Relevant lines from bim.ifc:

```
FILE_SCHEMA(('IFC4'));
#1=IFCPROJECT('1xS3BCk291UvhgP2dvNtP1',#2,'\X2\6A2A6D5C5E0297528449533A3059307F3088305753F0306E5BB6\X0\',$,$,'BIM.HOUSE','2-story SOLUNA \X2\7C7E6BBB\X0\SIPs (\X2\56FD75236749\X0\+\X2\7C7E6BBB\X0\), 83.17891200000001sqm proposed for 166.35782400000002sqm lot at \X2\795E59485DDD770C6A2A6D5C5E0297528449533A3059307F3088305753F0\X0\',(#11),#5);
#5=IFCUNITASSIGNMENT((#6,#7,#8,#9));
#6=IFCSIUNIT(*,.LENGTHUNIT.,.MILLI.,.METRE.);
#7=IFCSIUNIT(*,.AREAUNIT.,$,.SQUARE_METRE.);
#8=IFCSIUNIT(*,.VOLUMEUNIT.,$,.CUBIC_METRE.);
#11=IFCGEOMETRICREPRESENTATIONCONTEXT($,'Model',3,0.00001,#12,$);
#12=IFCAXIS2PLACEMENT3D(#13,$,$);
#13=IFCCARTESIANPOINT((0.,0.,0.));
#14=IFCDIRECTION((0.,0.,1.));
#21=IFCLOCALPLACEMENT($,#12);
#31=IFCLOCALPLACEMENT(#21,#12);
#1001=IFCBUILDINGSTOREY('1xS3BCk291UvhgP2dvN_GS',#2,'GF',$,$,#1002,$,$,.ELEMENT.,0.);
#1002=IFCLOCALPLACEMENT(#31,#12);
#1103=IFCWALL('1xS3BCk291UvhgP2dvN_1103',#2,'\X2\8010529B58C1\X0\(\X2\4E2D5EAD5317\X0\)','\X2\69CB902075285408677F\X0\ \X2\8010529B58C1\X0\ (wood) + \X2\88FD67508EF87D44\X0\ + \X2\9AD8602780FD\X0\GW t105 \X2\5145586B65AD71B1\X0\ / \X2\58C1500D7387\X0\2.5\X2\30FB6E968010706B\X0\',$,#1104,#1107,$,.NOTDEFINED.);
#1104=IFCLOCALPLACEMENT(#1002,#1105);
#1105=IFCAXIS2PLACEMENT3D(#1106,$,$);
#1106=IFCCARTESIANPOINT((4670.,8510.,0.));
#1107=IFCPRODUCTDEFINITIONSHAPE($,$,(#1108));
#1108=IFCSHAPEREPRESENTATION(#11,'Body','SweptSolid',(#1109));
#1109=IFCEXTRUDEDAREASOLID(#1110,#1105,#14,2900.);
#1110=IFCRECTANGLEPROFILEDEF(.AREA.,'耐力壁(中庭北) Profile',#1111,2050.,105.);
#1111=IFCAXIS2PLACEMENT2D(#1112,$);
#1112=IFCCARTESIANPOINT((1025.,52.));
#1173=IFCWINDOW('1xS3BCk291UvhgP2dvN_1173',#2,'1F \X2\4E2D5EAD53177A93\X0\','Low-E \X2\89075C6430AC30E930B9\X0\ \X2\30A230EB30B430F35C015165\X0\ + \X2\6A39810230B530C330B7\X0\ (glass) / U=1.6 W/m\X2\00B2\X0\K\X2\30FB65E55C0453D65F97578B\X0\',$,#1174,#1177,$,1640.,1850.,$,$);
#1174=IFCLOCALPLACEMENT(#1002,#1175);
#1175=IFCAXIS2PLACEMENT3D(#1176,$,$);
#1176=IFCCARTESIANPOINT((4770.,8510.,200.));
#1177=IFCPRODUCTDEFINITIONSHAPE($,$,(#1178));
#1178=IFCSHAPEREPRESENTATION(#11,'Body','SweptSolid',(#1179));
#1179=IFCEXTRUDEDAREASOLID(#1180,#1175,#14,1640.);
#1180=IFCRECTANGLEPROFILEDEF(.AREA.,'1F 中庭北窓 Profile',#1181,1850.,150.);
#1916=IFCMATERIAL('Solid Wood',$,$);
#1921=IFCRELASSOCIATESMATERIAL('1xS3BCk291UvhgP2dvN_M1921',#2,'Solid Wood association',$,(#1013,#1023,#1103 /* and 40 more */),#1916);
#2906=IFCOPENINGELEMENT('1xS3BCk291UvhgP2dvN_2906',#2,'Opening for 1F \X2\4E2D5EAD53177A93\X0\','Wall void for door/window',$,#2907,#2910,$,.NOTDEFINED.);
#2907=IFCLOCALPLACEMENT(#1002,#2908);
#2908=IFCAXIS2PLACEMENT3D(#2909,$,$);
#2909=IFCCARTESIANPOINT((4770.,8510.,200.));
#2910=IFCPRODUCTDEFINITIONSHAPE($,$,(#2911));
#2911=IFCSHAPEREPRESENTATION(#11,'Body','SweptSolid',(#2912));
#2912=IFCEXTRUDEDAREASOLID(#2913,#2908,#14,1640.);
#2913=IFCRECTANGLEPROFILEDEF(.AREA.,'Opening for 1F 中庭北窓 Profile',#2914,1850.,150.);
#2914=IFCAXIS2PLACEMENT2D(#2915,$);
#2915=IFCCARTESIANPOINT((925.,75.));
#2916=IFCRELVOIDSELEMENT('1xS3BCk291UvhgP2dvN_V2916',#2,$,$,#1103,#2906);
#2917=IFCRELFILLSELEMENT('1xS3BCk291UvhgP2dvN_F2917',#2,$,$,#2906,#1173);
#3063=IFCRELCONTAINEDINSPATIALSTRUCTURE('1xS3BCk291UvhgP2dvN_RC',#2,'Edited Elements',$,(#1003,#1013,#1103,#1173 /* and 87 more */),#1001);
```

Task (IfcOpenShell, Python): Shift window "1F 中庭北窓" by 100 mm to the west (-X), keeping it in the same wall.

```python
import ifcopenshell
import ifcopenshell.api.geometry
import ifcopenshell.util.placement
import ifcopenshell.util.unit

model = ifcopenshell.open("bim.ifc")
unit_scale = ifcopenshell.util.unit.calculate_unit_scale(model)

window = model.by_guid("1xS3BCk291UvhgP2dvN_1173")
opening = window.FillsVoids[0].RelatingOpeningElement
wall = opening.VoidsElements[0].RelatingBuildingElement

wall_matrix = ifcopenshell.util.placement.get_local_placement(wall.ObjectPlacement)
shift = wall_matrix[:3, 0] * -0.1 / unit_scale
before = ifcopenshell.util.placement.get_local_placement(window.ObjectPlacement)[:3, 3].copy()

# The window is not placed relative to its opening, so move both.
for product in (opening, window):
    matrix = ifcopenshell.util.placement.get_local_placement(product.ObjectPlacement)
    matrix[:3, 3] += shift
    ifcopenshell.api.geometry.edit_object_placement(model, product=product, matrix=matrix, is_si=False)

after = ifcopenshell.util.placement.get_local_placement(window.ObjectPlacement)[:3, 3]
print("window moved by", (after - before).round(3) + 0.0)

model.write("bim_v2.ifc")
```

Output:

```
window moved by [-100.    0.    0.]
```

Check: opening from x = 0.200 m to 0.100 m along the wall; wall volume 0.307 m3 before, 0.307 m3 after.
